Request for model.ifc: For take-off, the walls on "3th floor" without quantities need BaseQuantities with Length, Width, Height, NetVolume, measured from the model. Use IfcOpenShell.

First a look at what the model holds.

```python
import ifcopenshell
import ifcopenshell.util.element
import ifcopenshell.util.unit

model = ifcopenshell.open("model.ifc")
print(model.schema)
for unit_type in ("LENGTHUNIT", "AREAUNIT", "VOLUMEUNIT"):
    print(unit_type, ifcopenshell.util.unit.calculate_unit_scale(model, unit_type))
storey = next(s for s in model.by_type("IfcBuildingStorey") if s.Name == "3th floor")
walls = [e for e in ifcopenshell.util.element.get_decomposition(storey) if e.is_a("IfcWall")]
for e in sorted(walls, key=lambda e: e.id()):
    print(e.id(), e.is_a(), e.Name, list(ifcopenshell.util.element.get_psets(e, qtos_only=True)), sep=" | ")
```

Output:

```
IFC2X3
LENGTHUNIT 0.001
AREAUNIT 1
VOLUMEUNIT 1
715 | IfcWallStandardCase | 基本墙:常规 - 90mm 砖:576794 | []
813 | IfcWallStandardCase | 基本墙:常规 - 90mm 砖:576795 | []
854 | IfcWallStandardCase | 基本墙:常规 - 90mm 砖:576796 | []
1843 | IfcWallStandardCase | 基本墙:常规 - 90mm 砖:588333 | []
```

```python
import ifcopenshell
import ifcopenshell.api.pset
import ifcopenshell.geom
import ifcopenshell.util.element
import ifcopenshell.util.shape
import ifcopenshell.util.unit

model = ifcopenshell.open("model.ifc")
unit_scale = ifcopenshell.util.unit.calculate_unit_scale(model)
volume_scale = ifcopenshell.util.unit.calculate_unit_scale(model, "VOLUMEUNIT")
settings = ifcopenshell.geom.settings()

storey = next(s for s in model.by_type("IfcBuildingStorey") if s.Name == "3th floor")
walls = [e for e in ifcopenshell.util.element.get_decomposition(storey) if e.is_a("IfcWall")]

for e in sorted(walls, key=lambda e: e.id()):
    if ifcopenshell.util.element.get_psets(e, qtos_only=True, should_inherit=False):
        continue
    # Geometry comes back in metres, in the element's own axes.
    shape = ifcopenshell.geom.create_shape(settings, e)
    values = {
        "Length": ifcopenshell.util.shape.get_x(shape.geometry) / unit_scale,
        "Width": ifcopenshell.util.shape.get_y(shape.geometry) / unit_scale,
        "Height": ifcopenshell.util.shape.get_z(shape.geometry) / unit_scale,
        "NetVolume": ifcopenshell.util.shape.get_volume(shape.geometry) / volume_scale,
    }
    qto = ifcopenshell.api.pset.add_qto(model, product=e, name="BaseQuantities")
    ifcopenshell.api.pset.edit_qto(model, qto=qto, properties=values)
    print(e.id(), {k: round(v, 3) for k, v in values.items()})

model.write("model-out.ifc")
```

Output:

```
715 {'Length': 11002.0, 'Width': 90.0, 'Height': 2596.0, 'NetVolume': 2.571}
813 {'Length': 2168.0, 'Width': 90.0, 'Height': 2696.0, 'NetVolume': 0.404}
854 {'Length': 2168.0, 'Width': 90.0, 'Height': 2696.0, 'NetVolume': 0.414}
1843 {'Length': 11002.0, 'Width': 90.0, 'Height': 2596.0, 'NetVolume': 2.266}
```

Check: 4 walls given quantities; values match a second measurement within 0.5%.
